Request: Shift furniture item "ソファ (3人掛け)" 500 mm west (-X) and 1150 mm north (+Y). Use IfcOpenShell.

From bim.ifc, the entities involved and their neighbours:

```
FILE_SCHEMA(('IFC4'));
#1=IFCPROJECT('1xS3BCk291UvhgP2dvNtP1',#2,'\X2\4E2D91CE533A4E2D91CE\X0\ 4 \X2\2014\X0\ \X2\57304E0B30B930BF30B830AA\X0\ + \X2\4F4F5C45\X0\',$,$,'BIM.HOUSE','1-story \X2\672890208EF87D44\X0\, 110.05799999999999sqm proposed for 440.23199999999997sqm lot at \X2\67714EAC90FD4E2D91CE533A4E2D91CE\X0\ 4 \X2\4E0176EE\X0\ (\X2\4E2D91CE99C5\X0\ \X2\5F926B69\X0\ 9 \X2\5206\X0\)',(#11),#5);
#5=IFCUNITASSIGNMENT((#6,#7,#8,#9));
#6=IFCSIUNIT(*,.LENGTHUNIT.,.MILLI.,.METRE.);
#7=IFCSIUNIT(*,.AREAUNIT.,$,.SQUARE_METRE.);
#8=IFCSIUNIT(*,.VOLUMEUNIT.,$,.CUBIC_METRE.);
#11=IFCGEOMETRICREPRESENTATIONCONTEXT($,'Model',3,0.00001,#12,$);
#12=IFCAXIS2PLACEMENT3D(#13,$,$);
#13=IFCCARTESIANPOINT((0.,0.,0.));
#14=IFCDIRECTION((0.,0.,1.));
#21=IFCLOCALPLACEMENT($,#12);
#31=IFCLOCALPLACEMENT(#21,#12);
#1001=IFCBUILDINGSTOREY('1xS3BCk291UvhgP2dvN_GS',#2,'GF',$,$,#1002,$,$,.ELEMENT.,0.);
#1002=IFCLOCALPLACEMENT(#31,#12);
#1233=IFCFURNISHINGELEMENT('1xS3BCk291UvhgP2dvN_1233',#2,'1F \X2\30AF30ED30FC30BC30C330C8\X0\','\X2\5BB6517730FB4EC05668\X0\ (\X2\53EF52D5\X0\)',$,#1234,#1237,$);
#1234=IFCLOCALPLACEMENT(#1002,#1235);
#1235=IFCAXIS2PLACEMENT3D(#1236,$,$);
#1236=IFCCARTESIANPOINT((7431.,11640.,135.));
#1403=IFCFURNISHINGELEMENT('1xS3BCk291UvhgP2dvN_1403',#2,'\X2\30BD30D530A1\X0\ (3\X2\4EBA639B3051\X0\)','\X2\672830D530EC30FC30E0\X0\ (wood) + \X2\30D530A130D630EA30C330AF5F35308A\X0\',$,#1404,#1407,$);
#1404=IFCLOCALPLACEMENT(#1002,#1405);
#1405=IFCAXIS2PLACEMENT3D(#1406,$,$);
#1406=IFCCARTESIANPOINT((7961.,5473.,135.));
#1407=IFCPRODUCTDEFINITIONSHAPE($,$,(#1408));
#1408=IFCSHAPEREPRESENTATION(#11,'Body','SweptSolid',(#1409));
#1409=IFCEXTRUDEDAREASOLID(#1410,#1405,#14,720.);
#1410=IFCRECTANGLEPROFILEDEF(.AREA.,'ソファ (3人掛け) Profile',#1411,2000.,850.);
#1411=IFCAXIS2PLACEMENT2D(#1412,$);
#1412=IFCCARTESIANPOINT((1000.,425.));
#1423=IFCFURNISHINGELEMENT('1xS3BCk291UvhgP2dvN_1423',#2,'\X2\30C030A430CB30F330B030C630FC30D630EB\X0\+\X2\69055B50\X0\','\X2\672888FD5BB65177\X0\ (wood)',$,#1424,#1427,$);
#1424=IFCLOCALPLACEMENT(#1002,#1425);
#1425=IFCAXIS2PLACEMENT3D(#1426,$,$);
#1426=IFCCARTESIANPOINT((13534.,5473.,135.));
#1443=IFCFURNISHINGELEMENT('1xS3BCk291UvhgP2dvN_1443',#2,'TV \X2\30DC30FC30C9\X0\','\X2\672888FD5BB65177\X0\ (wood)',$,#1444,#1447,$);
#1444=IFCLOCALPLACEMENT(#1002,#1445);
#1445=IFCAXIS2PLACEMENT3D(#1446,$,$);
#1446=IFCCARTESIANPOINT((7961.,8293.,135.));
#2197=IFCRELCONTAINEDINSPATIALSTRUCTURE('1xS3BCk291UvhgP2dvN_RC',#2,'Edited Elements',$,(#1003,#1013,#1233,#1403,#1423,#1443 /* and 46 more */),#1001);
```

```python
import ifcopenshell
import ifcopenshell.api.geometry
import ifcopenshell.util.placement
import ifcopenshell.util.unit

model = ifcopenshell.open("bim.ifc")
unit_scale = ifcopenshell.util.unit.calculate_unit_scale(model)

item = model.by_guid("1xS3BCk291UvhgP2dvN_1403")
matrix = ifcopenshell.util.placement.get_local_placement(item.ObjectPlacement)
matrix[0, 3] -= 0.5 / unit_scale
matrix[1, 3] += 1.15 / unit_scale
ifcopenshell.api.geometry.edit_object_placement(model, product=item, matrix=matrix, is_si=False)

print(ifcopenshell.util.placement.get_local_placement(item.ObjectPlacement).round(3) + 0.0)

model.write("bim_v2.ifc")
```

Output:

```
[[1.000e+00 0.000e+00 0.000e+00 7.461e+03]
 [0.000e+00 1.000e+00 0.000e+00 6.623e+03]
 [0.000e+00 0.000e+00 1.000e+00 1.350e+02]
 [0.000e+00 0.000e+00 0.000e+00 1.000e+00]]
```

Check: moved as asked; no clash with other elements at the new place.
